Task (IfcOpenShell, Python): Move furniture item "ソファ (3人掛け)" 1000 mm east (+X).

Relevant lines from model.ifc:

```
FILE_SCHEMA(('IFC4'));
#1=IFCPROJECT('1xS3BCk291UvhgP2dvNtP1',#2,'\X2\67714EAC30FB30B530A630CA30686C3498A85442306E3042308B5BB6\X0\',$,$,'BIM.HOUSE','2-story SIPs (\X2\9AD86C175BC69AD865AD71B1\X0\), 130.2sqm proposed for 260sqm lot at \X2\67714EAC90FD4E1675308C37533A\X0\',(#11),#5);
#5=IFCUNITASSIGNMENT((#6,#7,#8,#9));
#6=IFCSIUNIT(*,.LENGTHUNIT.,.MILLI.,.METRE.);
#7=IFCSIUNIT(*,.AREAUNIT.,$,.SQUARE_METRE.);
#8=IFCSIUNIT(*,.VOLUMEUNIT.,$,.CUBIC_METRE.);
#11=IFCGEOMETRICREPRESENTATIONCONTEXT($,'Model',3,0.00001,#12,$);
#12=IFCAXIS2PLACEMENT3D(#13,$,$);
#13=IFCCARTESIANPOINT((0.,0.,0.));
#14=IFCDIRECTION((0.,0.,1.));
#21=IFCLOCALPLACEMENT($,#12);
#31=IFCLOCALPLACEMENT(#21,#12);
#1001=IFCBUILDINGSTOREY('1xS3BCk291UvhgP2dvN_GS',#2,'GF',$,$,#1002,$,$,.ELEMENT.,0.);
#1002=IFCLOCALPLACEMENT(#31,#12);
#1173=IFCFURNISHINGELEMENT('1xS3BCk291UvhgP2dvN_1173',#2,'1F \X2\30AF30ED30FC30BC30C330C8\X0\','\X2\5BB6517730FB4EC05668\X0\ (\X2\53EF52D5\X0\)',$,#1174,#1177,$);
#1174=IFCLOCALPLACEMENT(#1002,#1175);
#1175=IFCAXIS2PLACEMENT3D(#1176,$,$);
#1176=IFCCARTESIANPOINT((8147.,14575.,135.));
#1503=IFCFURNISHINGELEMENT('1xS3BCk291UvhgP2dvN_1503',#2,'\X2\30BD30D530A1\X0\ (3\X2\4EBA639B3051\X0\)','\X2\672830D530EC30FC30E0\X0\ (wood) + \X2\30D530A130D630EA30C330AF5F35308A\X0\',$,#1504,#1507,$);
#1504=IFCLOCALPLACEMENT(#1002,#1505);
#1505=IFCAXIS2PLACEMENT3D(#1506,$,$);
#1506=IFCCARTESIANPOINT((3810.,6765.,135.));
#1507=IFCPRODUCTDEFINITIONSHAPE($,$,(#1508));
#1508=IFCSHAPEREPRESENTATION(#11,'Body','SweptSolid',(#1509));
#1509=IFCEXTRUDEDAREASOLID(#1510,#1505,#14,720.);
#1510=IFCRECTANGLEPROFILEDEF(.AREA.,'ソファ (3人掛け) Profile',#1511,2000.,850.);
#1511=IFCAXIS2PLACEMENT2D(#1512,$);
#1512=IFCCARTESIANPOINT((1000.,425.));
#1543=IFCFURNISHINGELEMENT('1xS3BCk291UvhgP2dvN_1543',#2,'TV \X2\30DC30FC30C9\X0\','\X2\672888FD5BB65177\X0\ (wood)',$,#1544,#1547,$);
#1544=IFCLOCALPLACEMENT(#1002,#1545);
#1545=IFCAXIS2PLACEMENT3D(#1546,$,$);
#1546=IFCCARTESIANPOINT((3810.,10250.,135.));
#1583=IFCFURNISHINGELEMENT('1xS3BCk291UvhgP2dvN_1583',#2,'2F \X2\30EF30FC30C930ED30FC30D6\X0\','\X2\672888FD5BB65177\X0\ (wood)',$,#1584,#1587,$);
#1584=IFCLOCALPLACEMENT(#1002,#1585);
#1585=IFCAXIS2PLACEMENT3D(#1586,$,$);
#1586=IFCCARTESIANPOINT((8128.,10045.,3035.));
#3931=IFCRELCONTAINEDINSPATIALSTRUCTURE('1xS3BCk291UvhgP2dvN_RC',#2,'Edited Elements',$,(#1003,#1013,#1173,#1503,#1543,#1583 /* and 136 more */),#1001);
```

```python
import ifcopenshell
import ifcopenshell.api.geometry
import ifcopenshell.util.placement

model = ifcopenshell.open("model.ifc")

item = model.by_guid("1xS3BCk291UvhgP2dvN_1503")
matrix = ifcopenshell.util.placement.get_local_placement(item.ObjectPlacement)
matrix[0, 3] += 1000.0
ifcopenshell.api.geometry.edit_object_placement(model, product=item, matrix=matrix, is_si=False)

print(ifcopenshell.util.placement.get_local_placement(item.ObjectPlacement).round(3) + 0.0)

model.write("model_rev.ifc")
```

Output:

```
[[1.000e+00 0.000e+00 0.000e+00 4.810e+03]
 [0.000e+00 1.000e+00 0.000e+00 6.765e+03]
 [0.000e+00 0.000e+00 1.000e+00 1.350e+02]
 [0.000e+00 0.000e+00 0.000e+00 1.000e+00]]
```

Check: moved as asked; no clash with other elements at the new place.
